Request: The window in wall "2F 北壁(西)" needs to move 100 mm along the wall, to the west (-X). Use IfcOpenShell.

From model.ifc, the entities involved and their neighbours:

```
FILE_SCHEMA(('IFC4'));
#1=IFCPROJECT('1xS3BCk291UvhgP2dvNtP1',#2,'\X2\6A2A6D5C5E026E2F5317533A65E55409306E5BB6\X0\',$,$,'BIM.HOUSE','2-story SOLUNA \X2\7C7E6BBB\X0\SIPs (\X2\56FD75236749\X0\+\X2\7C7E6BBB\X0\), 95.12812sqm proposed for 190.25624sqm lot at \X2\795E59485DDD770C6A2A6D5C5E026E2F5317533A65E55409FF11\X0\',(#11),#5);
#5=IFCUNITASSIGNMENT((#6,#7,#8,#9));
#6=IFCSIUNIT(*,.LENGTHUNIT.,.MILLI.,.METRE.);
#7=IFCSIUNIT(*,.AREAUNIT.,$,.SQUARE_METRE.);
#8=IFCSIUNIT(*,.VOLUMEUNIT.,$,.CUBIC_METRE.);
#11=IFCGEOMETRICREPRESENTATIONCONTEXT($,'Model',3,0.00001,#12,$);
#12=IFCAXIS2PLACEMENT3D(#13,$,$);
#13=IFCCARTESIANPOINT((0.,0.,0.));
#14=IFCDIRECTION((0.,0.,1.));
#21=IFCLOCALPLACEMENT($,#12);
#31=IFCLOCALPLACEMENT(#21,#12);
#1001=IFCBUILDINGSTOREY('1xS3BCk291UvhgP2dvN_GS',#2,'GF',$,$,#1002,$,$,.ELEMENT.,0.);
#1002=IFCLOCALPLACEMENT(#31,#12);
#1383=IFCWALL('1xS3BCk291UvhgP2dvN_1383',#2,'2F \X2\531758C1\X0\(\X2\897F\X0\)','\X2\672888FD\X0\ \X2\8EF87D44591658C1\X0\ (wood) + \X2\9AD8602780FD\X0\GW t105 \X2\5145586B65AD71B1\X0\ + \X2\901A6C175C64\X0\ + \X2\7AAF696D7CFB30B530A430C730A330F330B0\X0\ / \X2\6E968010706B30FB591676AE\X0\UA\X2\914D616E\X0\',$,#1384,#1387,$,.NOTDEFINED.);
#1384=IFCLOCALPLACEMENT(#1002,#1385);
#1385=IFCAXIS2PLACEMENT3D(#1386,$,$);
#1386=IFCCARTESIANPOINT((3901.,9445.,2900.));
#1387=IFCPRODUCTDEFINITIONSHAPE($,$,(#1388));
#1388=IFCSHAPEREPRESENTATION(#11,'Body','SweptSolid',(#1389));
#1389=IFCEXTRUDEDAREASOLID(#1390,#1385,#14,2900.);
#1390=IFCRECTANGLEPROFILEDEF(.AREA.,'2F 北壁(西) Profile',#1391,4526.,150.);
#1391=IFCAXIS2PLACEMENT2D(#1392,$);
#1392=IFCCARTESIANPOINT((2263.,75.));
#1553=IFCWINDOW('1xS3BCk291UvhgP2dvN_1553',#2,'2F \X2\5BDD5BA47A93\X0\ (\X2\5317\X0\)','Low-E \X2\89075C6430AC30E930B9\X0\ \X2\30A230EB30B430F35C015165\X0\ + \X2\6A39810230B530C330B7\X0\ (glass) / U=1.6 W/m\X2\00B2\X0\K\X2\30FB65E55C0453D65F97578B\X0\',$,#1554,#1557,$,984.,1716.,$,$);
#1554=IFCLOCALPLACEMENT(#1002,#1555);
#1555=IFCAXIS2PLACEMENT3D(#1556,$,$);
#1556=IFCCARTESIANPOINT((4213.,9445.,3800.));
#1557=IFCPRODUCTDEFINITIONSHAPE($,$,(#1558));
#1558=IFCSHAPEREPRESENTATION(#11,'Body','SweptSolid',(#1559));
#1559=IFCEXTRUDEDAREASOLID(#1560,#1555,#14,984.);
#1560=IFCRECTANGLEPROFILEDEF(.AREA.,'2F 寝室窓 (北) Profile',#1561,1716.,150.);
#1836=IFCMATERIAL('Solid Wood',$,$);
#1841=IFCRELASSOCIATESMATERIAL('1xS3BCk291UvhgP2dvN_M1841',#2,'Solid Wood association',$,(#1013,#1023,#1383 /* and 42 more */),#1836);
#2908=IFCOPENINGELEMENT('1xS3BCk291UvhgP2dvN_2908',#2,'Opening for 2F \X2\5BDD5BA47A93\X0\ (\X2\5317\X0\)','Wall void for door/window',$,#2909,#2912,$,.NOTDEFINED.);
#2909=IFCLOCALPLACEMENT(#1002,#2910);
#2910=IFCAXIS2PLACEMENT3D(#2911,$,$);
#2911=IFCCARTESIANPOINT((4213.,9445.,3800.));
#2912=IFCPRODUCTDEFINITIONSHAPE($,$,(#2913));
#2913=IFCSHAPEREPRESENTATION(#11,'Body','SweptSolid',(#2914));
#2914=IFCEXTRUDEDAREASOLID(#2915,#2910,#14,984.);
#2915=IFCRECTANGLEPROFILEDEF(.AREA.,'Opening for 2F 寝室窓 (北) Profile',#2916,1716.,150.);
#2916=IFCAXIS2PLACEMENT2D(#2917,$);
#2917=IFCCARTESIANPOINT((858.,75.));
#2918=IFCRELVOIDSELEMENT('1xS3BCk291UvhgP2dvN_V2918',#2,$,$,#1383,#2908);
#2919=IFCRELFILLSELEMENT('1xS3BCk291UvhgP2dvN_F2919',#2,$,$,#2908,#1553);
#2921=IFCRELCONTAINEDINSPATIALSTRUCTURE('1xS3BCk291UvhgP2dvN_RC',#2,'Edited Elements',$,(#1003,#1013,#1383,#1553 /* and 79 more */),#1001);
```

```python
import ifcopenshell
import ifcopenshell.api.geometry
import ifcopenshell.util.placement
import ifcopenshell.util.unit

model = ifcopenshell.open("model.ifc")
unit_scale = ifcopenshell.util.unit.calculate_unit_scale(model)

window = model.by_id(1553)
opening = window.FillsVoids[0].RelatingOpeningElement
wall = opening.VoidsElements[0].RelatingBuildingElement

wall_matrix = ifcopenshell.util.placement.get_local_placement(wall.ObjectPlacement)
shift = wall_matrix[:3, 0] * -0.1 / unit_scale
before = ifcopenshell.util.placement.get_local_placement(window.ObjectPlacement)[:3, 3].copy()

# The window is not placed relative to its opening, so move both.
for product in (opening, window):
    matrix = ifcopenshell.util.placement.get_local_placement(product.ObjectPlacement)
    matrix[:3, 3] += shift
    ifcopenshell.api.geometry.edit_object_placement(model, product=product, matrix=matrix, is_si=False)

after = ifcopenshell.util.placement.get_local_placement(window.ObjectPlacement)[:3, 3]
print("window moved by", (after - before).round(3) + 0.0)

model.write("model_rev.ifc")
```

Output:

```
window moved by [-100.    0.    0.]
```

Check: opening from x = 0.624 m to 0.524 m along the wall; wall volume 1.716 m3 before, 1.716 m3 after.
